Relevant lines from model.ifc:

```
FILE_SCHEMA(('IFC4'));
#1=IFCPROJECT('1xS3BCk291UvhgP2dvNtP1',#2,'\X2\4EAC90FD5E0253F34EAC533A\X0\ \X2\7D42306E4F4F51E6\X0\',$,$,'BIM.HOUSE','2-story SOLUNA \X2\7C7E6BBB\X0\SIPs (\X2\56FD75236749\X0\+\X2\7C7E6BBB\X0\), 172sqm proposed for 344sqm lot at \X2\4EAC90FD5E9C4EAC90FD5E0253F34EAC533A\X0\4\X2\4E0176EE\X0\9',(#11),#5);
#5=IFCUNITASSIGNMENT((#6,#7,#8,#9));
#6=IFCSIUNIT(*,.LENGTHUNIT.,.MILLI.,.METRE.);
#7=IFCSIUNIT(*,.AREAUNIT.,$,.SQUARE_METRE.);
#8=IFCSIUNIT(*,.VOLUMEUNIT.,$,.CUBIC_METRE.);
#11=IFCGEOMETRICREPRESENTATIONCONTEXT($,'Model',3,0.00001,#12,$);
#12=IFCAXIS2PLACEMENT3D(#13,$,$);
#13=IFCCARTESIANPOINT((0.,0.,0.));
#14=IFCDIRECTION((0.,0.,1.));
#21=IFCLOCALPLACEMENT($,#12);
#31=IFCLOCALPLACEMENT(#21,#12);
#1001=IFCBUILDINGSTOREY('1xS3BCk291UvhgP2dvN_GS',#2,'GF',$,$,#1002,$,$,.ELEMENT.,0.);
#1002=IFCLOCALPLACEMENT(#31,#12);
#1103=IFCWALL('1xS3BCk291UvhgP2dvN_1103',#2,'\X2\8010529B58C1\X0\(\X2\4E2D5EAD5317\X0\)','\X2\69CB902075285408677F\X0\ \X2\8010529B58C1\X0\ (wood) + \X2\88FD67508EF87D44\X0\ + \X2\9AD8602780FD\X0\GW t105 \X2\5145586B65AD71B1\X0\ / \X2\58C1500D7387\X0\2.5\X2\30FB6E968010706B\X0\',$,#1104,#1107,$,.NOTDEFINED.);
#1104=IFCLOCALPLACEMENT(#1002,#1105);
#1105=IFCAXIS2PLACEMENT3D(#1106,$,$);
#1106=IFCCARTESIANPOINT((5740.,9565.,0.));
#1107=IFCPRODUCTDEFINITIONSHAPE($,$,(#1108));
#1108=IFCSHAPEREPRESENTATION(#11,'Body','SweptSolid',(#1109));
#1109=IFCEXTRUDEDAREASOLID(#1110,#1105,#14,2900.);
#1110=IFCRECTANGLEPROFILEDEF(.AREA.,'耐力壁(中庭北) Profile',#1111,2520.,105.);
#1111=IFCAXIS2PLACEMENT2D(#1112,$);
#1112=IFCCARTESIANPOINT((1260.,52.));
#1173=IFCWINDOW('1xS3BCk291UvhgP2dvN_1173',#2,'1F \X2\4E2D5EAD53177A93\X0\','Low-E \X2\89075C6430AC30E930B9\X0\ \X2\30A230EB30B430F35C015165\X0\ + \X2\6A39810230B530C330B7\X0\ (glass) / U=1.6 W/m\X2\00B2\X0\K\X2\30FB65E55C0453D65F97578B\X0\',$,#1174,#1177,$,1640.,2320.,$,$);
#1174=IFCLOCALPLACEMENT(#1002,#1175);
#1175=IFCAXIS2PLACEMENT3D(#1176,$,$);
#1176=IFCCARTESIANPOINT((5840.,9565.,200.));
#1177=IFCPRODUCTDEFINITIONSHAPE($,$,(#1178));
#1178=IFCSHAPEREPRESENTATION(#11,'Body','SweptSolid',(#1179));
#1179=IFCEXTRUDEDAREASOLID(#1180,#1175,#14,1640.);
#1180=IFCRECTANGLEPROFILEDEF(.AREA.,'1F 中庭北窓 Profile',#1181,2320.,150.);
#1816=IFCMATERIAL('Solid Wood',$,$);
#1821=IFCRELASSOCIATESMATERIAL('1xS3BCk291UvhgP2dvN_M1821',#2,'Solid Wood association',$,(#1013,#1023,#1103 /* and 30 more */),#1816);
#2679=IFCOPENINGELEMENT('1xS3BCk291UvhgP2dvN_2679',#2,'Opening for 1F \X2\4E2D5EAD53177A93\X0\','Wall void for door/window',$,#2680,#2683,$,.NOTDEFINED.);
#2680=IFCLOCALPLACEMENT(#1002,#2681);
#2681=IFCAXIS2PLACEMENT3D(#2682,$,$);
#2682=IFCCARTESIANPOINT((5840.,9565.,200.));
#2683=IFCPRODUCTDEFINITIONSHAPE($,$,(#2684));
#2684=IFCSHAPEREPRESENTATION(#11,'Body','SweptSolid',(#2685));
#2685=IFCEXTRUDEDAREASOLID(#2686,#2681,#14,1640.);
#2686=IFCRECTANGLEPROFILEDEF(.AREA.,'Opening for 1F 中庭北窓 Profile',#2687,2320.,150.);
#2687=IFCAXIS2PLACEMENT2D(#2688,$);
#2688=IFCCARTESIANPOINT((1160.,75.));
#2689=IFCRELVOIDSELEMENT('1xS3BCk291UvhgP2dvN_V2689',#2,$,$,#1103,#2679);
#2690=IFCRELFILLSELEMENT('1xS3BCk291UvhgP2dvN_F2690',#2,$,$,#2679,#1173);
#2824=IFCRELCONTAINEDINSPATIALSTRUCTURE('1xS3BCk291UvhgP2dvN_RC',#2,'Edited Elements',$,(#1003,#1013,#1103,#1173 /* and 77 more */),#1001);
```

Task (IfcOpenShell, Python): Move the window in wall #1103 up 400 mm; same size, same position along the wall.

```python
import numpy as np
import ifcopenshell
import ifcopenshell.api.geometry
import ifcopenshell.util.placement
import ifcopenshell.util.unit

model = ifcopenshell.open("model.ifc")
unit_scale = ifcopenshell.util.unit.calculate_unit_scale(model)

window = model.by_id(1173)
opening = window.FillsVoids[0].RelatingOpeningElement
dz = 0.4 / unit_scale

shift = np.array([0.0, 0.0, dz])
# The window is not placed relative to its opening, so move both.
for product in (opening, window):
    matrix = ifcopenshell.util.placement.get_local_placement(product.ObjectPlacement)
    matrix[:3, 3] += shift
    ifcopenshell.api.geometry.edit_object_placement(model, product=product, matrix=matrix, is_si=False)

print(f"moved by {dz * unit_scale:+.3f} m")

model.write("model-out.ifc")
```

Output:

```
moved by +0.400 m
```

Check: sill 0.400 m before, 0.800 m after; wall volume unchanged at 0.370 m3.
